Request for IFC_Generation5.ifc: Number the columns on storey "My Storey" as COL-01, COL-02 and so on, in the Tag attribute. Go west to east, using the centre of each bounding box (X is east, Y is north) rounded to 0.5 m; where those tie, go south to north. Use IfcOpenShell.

First a look at what the model holds.

```python
import ifcopenshell
import ifcopenshell.util.element
import ifcopenshell.util.placement

model = ifcopenshell.open("IFC_Generation5.ifc")
print(model.schema)
storey = next(s for s in model.by_type("IfcBuildingStorey") if s.Name == "My Storey")
columns = [e for e in ifcopenshell.util.element.get_decomposition(storey) if e.is_a("IfcColumn")]
for e in sorted(columns, key=lambda e: e.id()):
    origin = ifcopenshell.util.placement.get_local_placement(e.ObjectPlacement)[:3, 3]
    print(e.id(), e.Tag, e.Name, origin.round(2) + 0.0, sep=" | ")
```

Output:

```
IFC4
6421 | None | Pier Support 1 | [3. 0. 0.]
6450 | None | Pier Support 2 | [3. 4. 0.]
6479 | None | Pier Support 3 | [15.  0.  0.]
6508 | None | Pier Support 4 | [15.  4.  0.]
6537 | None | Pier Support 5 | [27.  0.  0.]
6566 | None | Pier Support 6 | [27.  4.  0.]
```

```python
import ifcopenshell
import ifcopenshell.geom
import ifcopenshell.util.element
import ifcopenshell.util.shape

model = ifcopenshell.open("IFC_Generation5.ifc")
settings = ifcopenshell.geom.settings()
settings.set("use-world-coords", True)


def centre(element):
    shape = ifcopenshell.geom.create_shape(settings, element)
    return ifcopenshell.util.shape.get_bbox_centroid(shape.geometry)


storey = next(s for s in model.by_type("IfcBuildingStorey") if s.Name == "My Storey")
columns = [e for e in ifcopenshell.util.element.get_decomposition(storey) if e.is_a("IfcColumn")]

# Insertion points can sit at a corner or the storey origin, so sort by the geometry (in metres).
centres = {e: centre(e) for e in columns}
columns.sort(key=lambda e: (round(centres[e][0] / 0.5), centres[e][1]))

for i, e in enumerate(columns, start=1):
    number = f"COL-{i:02d}"
    e.Tag = number
    print(e.id(), number)

model.write("IFC_Generation5-out.ifc")
```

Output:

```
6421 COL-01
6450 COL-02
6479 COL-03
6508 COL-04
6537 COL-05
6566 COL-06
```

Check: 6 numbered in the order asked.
